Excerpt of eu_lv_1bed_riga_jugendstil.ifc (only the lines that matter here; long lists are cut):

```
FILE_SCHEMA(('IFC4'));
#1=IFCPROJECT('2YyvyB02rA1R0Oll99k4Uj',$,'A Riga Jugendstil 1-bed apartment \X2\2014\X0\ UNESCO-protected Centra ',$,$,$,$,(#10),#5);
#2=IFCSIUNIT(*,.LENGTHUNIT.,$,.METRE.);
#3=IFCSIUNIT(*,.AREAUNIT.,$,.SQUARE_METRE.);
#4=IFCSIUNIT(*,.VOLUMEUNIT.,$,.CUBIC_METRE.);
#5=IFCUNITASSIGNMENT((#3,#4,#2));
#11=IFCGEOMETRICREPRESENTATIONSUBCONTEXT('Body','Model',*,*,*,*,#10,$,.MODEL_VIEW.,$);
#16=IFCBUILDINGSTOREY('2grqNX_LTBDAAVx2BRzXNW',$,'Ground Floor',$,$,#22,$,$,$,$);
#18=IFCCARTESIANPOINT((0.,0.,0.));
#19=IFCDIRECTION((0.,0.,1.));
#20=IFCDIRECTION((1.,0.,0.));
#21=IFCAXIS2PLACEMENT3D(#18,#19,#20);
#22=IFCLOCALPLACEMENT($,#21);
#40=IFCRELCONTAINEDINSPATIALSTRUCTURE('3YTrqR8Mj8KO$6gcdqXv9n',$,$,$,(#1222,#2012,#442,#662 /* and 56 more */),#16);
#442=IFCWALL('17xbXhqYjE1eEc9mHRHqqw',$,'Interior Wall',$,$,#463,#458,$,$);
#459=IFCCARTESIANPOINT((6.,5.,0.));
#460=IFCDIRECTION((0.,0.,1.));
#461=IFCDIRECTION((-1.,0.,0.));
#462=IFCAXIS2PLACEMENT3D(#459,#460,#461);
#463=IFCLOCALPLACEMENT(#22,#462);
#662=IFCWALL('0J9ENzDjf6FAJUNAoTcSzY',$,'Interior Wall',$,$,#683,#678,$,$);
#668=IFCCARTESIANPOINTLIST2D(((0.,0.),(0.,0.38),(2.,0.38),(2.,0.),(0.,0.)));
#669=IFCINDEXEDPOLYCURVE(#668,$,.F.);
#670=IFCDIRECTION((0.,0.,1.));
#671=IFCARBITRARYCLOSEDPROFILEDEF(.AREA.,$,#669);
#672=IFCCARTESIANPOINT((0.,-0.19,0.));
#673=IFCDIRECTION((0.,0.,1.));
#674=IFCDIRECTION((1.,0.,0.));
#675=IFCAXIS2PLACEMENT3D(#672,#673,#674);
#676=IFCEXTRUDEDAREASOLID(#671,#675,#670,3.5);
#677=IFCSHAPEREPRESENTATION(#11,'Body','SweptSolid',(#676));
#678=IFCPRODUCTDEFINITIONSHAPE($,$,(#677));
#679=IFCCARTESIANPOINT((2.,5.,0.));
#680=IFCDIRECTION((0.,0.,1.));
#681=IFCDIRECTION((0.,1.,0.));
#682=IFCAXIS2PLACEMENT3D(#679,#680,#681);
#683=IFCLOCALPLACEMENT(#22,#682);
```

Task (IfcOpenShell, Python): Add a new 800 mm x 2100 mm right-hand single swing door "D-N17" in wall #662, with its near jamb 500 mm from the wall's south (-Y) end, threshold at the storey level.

```python
import numpy as np
import ifcopenshell
import ifcopenshell.api.feature
import ifcopenshell.api.geometry
import ifcopenshell.api.root
import ifcopenshell.api.spatial
import ifcopenshell.geom
import ifcopenshell.util.element
import ifcopenshell.util.placement
import ifcopenshell.util.representation
import ifcopenshell.util.shape
import ifcopenshell.util.unit

model = ifcopenshell.open("eu_lv_1bed_riga_jugendstil.ifc")
unit_scale = ifcopenshell.util.unit.calculate_unit_scale(model)
settings = ifcopenshell.geom.settings()


def volume(element):
    """Net volume in cubic metres, openings subtracted."""
    shape = ifcopenshell.geom.create_shape(settings, element)
    return ifcopenshell.util.shape.get_volume(shape.geometry)


wall = model.by_guid("0J9ENzDjf6FAJUNAoTcSzY")
storey = ifcopenshell.util.element.get_container(wall, ifc_class="IfcBuildingStorey")
context = ifcopenshell.util.representation.get_context(model, "Model", "Body", "MODEL_VIEW")
before = volume(wall)

width, height, from_end, sill = 0.8, 2.1, 0.5, 0.0  # metres

# The wall runs along its own X axis, and the end named is its -X end.
wall_shape = ifcopenshell.geom.create_shape(settings, wall)
x, y, z = ifcopenshell.util.shape.get_vertices(wall_shape.geometry).T
start = x.min() + from_end
face, thickness = float(y.min()), float(y.max() - y.min())
wall_matrix = ifcopenshell.util.placement.get_local_placement(wall.ObjectPlacement)
level = ifcopenshell.util.placement.get_local_placement(storey.ObjectPlacement)[2, 3]


def in_wall(x, y):
    """Placement at x, y metres in the wall's axes, at sill height."""
    matrix = wall_matrix.copy()
    matrix[:, 3] = wall_matrix @ np.array([x / unit_scale, y / unit_scale, 0.0, 1.0])
    matrix[2, 3] = level + sill / unit_scale
    return matrix


# Opening: a box that overshoots both wall faces by 50 mm.
opening = ifcopenshell.api.root.create_entity(model, ifc_class="IfcOpeningElement", predefined_type="OPENING")
box = ifcopenshell.api.geometry.add_wall_representation(
    model, context=context, length=width, height=height, thickness=thickness + 0.1
)
ifcopenshell.api.geometry.assign_representation(model, product=opening, representation=box)
ifcopenshell.api.geometry.edit_object_placement(model, product=opening, matrix=in_wall(start, face - 0.05), is_si=False)
ifcopenshell.api.feature.add_feature(model, feature=opening, element=wall)

door = ifcopenshell.api.root.create_entity(model, ifc_class="IfcDoor", name="D-N17", predefined_type="DOOR")
door.OverallWidth, door.OverallHeight = width / unit_scale, height / unit_scale
door.OperationType = "SINGLE_SWING_RIGHT"
body = ifcopenshell.api.geometry.add_door_representation(
    model,
    context=context,
    overall_width=door.OverallWidth,
    overall_height=door.OverallHeight,
    operation_type="SINGLE_SWING_RIGHT",
    lining_properties={"LiningDepth": thickness / unit_scale, "ThresholdDepth": thickness / unit_scale},
)
ifcopenshell.api.geometry.assign_representation(model, product=door, representation=body)
ifcopenshell.api.spatial.assign_container(model, products=[door], relating_structure=storey)
ifcopenshell.api.feature.add_filling(model, opening=opening, element=door)

# The lining spans the wall, so the door starts at the wall face.
ifcopenshell.api.geometry.edit_object_placement(model, product=door, matrix=in_wall(start, face), is_si=False)

after = volume(wall)

print(f"wall volume {before:.3f} -> {after:.3f} m3")

model.write("eu_lv_1bed_riga_jugendstil_rev.ifc")
```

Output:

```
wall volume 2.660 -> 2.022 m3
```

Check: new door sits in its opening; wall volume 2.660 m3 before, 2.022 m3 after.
